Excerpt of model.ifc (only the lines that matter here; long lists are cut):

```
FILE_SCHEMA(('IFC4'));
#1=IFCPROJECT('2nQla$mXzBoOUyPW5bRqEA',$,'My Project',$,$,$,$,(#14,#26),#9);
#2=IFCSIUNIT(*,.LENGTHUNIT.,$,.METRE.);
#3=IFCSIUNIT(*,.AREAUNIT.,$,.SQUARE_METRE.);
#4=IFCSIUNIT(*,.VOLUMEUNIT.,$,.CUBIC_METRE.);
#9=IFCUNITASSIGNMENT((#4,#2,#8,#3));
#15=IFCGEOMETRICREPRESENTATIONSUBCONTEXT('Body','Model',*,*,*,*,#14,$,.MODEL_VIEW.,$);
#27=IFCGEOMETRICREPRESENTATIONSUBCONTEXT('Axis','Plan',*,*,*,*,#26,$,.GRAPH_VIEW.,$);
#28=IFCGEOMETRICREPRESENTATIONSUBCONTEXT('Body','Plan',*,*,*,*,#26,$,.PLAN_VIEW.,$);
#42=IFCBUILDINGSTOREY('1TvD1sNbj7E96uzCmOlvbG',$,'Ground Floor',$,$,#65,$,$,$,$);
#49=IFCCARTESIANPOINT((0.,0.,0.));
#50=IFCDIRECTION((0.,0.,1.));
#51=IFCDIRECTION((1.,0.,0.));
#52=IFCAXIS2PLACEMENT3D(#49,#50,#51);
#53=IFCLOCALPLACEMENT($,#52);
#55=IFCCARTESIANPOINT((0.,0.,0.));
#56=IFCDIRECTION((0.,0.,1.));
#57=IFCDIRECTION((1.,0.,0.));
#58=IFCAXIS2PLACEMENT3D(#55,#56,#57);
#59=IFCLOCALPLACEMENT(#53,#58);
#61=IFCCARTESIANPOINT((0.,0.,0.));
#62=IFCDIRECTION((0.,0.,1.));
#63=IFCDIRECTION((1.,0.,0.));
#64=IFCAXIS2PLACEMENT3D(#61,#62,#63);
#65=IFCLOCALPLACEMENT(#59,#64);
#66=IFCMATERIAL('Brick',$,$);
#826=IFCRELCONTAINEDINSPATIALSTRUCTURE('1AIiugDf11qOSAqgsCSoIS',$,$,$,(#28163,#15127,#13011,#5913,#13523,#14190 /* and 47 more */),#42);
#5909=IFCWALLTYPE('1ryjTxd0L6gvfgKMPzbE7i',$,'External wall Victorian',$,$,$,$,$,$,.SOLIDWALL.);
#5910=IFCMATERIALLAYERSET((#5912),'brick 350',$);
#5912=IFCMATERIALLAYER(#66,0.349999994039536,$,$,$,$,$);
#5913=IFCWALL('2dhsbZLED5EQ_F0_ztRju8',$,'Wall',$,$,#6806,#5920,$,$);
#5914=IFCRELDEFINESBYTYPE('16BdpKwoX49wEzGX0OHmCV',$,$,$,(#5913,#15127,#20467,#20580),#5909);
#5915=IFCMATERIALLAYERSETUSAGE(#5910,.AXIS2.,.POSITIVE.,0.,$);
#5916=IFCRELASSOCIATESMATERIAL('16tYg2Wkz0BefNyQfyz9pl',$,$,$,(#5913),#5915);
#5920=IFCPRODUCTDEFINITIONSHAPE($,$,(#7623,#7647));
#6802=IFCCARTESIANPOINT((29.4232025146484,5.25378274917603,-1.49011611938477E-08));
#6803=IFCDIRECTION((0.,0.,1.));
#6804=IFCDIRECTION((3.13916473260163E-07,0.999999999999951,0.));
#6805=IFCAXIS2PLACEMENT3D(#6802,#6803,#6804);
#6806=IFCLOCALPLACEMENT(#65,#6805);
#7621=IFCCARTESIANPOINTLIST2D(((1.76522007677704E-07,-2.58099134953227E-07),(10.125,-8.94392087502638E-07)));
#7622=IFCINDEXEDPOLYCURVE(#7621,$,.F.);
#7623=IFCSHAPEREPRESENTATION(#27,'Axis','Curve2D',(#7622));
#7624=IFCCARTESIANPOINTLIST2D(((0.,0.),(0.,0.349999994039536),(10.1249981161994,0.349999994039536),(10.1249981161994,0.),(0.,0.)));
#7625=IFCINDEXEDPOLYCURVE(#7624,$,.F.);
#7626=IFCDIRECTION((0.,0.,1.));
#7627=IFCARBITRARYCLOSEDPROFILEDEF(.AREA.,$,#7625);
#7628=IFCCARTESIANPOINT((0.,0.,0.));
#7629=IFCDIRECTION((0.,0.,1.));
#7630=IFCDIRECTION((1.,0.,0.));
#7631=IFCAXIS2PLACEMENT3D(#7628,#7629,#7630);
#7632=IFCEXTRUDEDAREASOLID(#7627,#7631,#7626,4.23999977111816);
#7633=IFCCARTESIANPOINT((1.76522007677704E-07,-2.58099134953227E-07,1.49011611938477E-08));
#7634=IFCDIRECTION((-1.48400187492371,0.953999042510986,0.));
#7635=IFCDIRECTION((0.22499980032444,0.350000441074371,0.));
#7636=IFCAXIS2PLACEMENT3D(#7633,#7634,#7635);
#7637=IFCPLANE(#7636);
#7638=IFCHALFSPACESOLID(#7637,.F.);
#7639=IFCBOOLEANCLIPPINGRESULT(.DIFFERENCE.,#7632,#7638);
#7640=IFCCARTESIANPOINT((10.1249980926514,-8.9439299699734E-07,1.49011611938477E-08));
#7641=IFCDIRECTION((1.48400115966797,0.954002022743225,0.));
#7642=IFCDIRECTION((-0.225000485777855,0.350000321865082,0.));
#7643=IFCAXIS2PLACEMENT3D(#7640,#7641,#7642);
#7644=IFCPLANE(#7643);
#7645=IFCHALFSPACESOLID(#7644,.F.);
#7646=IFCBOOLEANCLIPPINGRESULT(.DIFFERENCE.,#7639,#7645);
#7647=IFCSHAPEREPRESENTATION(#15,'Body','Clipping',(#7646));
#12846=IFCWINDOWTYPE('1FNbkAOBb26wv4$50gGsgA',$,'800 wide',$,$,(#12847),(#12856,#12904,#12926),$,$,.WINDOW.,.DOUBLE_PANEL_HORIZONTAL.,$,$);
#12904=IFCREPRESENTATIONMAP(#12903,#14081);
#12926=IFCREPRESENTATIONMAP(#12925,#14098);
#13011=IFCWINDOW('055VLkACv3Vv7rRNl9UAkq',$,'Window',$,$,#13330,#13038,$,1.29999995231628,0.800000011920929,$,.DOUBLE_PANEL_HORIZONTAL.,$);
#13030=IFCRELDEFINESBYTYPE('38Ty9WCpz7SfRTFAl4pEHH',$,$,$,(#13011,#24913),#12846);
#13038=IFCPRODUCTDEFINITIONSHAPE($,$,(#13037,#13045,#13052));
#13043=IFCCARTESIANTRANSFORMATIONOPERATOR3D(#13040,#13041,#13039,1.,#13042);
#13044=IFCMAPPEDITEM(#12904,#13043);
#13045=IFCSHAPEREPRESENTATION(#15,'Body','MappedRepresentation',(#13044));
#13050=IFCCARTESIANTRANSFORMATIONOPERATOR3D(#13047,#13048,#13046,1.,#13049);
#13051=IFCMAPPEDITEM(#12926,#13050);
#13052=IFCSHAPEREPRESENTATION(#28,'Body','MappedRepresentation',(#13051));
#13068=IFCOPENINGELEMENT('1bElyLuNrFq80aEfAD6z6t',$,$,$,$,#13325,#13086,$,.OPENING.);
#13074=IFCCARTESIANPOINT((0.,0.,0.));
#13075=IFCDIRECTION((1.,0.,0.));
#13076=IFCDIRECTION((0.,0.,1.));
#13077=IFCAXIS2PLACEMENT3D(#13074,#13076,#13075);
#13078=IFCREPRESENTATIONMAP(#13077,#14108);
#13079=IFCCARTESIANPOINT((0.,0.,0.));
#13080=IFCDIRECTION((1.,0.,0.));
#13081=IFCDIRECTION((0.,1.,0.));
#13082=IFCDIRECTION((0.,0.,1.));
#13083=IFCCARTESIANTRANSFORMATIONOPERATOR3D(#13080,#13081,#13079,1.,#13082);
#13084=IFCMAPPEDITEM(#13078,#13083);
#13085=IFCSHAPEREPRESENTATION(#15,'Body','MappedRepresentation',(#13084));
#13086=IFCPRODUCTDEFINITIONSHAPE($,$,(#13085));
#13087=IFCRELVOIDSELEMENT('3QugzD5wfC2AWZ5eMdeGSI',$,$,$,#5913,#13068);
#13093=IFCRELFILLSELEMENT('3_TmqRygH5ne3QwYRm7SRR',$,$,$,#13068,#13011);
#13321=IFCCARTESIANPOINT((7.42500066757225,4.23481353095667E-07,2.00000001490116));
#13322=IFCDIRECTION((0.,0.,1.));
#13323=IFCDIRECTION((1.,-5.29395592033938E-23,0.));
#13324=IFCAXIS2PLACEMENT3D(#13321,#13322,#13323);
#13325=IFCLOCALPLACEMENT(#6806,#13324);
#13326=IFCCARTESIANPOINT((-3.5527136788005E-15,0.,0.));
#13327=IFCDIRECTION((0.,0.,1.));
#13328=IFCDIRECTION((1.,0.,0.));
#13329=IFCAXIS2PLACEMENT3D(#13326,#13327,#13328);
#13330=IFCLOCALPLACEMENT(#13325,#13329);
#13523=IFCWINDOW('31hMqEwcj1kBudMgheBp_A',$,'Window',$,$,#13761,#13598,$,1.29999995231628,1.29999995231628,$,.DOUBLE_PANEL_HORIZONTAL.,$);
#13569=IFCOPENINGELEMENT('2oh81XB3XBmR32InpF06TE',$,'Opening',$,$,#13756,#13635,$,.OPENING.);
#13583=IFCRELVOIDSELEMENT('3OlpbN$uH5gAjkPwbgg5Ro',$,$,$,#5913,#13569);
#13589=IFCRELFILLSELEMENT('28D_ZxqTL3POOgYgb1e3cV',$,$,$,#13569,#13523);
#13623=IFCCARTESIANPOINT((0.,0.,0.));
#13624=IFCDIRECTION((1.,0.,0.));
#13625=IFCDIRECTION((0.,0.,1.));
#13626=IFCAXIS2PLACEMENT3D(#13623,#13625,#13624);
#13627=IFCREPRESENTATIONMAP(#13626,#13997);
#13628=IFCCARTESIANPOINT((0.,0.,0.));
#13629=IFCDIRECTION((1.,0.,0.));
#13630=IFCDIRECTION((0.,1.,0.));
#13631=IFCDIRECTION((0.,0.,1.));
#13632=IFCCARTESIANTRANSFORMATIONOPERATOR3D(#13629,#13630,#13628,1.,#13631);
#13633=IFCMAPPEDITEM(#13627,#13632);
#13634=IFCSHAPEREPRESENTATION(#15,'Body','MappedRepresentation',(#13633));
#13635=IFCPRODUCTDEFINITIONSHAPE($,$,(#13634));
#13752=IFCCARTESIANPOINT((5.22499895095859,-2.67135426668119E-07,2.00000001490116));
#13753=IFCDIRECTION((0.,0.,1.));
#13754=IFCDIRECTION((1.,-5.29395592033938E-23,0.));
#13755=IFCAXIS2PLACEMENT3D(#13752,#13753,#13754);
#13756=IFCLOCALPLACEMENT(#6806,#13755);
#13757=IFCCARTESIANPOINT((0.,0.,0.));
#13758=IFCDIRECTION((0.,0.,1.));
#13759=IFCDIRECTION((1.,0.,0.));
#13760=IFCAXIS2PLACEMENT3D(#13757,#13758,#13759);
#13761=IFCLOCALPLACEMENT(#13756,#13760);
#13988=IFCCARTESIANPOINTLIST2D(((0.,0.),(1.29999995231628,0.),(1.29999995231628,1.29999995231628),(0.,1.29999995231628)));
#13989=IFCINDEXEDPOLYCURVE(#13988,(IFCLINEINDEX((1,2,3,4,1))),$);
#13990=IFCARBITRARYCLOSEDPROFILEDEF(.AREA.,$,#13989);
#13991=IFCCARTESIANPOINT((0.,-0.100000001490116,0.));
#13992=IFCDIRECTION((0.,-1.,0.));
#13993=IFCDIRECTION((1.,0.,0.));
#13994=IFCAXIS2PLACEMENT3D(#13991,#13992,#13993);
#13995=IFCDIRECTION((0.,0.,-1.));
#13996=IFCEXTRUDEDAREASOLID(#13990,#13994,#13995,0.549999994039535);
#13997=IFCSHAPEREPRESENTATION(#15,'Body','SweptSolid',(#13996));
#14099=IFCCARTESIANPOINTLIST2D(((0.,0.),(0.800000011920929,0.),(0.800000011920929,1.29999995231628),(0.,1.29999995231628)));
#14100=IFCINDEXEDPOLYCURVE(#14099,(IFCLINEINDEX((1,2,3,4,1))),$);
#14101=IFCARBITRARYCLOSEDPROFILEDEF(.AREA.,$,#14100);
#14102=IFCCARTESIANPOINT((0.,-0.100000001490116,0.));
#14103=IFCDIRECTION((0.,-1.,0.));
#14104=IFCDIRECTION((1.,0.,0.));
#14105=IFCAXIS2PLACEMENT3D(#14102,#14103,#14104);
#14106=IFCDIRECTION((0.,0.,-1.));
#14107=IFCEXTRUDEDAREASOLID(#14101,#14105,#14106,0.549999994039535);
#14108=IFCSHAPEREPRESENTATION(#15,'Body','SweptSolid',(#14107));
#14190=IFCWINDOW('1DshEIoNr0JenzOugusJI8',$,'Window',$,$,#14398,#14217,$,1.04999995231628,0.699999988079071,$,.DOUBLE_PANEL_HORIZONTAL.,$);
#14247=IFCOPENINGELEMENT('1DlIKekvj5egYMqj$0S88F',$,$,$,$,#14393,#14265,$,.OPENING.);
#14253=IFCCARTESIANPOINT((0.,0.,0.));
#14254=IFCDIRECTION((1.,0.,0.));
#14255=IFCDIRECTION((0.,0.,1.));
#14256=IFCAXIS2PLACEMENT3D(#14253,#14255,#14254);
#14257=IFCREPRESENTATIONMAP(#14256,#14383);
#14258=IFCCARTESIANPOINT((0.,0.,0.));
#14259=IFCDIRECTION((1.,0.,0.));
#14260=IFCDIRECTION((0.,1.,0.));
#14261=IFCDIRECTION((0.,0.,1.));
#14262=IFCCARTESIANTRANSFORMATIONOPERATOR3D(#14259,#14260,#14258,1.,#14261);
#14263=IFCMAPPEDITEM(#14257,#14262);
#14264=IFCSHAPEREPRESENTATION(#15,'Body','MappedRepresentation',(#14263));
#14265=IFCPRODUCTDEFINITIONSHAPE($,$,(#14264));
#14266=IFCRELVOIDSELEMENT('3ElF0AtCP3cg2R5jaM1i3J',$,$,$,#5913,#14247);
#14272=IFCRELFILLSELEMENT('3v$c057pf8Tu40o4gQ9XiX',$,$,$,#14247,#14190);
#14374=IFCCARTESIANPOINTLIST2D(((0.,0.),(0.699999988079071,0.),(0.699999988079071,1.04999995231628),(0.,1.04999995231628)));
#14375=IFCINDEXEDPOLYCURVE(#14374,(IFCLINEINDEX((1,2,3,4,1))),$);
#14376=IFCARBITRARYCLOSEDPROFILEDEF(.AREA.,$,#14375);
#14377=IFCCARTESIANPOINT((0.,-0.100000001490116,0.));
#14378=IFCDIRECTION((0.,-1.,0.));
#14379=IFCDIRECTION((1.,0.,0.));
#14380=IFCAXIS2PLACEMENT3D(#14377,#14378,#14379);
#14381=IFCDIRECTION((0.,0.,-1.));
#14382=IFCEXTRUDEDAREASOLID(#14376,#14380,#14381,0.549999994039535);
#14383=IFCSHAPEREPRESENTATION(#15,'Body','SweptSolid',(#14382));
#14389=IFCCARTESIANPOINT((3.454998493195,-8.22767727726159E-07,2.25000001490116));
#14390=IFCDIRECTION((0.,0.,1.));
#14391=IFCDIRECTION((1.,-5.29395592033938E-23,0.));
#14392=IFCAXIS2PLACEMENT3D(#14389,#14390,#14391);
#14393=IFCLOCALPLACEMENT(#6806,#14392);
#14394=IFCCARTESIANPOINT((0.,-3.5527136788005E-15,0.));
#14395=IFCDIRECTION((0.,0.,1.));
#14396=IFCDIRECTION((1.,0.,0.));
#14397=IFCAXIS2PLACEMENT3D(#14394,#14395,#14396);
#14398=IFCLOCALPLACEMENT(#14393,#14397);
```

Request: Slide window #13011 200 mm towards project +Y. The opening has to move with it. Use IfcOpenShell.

```python
import ifcopenshell
import ifcopenshell.api.geometry
import ifcopenshell.util.placement

model = ifcopenshell.open("model.ifc")

window = model.by_id(13011)
opening = window.FillsVoids[0].RelatingOpeningElement
wall = opening.VoidsElements[0].RelatingBuildingElement

wall_matrix = ifcopenshell.util.placement.get_local_placement(wall.ObjectPlacement)
shift = wall_matrix[:3, 0] * 0.2
before = ifcopenshell.util.placement.get_local_placement(window.ObjectPlacement)[:3, 3].copy()

# The window is placed relative to its opening, so it follows when the opening moves.
matrix = ifcopenshell.util.placement.get_local_placement(opening.ObjectPlacement)
matrix[:3, 3] += shift
ifcopenshell.api.geometry.edit_object_placement(
    model, product=opening, matrix=matrix, is_si=False, should_transform_children=True
)

after = ifcopenshell.util.placement.get_local_placement(window.ObjectPlacement)[:3, 3]
print("window moved by", (after - before).round(3) + 0.0)

model.write("model_updated.ifc")
```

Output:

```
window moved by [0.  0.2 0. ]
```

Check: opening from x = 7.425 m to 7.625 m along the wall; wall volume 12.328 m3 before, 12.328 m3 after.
